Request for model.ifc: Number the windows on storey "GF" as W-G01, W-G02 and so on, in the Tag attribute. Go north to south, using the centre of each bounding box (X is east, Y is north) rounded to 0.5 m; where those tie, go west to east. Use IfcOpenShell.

First a look at what the model holds.

```python
import ifcopenshell
import ifcopenshell.util.element
import ifcopenshell.util.placement

model = ifcopenshell.open("model.ifc")
print(model.schema)
storey = next(s for s in model.by_type("IfcBuildingStorey") if s.Name == "GF")
windows = [e for e in ifcopenshell.util.element.get_decomposition(storey) if e.is_a("IfcWindow")]
for e in sorted(windows, key=lambda e: e.id()):
    origin = ifcopenshell.util.placement.get_local_placement(e.ObjectPlacement)[:3, 3]
    print(e.id(), e.Tag, e.Name, origin.round(2) + 0.0, sep=" | ")
```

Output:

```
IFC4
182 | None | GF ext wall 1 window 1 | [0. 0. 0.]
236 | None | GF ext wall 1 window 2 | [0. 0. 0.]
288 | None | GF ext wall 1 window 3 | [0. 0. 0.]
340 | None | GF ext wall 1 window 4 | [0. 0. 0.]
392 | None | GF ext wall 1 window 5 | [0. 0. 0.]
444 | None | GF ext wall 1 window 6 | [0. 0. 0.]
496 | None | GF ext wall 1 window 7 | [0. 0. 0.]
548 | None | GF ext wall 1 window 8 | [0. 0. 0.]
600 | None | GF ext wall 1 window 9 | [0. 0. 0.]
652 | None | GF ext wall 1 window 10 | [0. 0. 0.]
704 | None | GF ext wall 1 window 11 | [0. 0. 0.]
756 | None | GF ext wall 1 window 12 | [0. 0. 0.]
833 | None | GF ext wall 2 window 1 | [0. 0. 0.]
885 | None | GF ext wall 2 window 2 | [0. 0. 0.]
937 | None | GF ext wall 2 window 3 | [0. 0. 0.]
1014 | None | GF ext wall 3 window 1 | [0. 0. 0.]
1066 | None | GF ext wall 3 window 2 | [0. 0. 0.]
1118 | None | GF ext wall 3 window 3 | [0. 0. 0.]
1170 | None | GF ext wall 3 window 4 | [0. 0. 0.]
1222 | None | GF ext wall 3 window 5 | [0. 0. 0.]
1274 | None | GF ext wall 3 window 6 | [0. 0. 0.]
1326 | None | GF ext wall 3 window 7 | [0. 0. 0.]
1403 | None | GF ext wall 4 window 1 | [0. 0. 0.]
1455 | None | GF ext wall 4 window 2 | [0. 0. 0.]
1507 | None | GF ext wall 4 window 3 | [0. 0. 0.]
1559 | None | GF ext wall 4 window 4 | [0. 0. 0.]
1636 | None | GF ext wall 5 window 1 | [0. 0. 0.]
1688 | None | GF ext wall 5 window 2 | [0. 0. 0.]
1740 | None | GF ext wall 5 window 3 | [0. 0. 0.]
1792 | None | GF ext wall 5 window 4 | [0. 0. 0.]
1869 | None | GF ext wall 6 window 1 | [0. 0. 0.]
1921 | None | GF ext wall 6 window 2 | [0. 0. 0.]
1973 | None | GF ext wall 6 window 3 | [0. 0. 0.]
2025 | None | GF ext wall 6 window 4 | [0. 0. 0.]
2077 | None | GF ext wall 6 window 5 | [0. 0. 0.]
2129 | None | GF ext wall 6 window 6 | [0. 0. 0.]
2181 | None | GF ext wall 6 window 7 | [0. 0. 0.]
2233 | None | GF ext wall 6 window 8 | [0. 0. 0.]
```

```python
import ifcopenshell
import ifcopenshell.geom
import ifcopenshell.util.element
import ifcopenshell.util.shape

model = ifcopenshell.open("model.ifc")
settings = ifcopenshell.geom.settings()
settings.set("use-world-coords", True)


def centre(element):
    shape = ifcopenshell.geom.create_shape(settings, element)
    return ifcopenshell.util.shape.get_bbox_centroid(shape.geometry)


storey = next(s for s in model.by_type("IfcBuildingStorey") if s.Name == "GF")
windows = [e for e in ifcopenshell.util.element.get_decomposition(storey) if e.is_a("IfcWindow")]

# Insertion points can sit at a corner or the storey origin, so sort by the geometry (in metres).
centres = {e: centre(e) for e in windows}
windows.sort(key=lambda e: (-round(centres[e][1] / 0.5), centres[e][0]))

for i, e in enumerate(windows, start=1):
    number = f"W-G{i:02d}"
    e.Tag = number
    print(e.id(), number)

model.write("model_updated.ifc")
```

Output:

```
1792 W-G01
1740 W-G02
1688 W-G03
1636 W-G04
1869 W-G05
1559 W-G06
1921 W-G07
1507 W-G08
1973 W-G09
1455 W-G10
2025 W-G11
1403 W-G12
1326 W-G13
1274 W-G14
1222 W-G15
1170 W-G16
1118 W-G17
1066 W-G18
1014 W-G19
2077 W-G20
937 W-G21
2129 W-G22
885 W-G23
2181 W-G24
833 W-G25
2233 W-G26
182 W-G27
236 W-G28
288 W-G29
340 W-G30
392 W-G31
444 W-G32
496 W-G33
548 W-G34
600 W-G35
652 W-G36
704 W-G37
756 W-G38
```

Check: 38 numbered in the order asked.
